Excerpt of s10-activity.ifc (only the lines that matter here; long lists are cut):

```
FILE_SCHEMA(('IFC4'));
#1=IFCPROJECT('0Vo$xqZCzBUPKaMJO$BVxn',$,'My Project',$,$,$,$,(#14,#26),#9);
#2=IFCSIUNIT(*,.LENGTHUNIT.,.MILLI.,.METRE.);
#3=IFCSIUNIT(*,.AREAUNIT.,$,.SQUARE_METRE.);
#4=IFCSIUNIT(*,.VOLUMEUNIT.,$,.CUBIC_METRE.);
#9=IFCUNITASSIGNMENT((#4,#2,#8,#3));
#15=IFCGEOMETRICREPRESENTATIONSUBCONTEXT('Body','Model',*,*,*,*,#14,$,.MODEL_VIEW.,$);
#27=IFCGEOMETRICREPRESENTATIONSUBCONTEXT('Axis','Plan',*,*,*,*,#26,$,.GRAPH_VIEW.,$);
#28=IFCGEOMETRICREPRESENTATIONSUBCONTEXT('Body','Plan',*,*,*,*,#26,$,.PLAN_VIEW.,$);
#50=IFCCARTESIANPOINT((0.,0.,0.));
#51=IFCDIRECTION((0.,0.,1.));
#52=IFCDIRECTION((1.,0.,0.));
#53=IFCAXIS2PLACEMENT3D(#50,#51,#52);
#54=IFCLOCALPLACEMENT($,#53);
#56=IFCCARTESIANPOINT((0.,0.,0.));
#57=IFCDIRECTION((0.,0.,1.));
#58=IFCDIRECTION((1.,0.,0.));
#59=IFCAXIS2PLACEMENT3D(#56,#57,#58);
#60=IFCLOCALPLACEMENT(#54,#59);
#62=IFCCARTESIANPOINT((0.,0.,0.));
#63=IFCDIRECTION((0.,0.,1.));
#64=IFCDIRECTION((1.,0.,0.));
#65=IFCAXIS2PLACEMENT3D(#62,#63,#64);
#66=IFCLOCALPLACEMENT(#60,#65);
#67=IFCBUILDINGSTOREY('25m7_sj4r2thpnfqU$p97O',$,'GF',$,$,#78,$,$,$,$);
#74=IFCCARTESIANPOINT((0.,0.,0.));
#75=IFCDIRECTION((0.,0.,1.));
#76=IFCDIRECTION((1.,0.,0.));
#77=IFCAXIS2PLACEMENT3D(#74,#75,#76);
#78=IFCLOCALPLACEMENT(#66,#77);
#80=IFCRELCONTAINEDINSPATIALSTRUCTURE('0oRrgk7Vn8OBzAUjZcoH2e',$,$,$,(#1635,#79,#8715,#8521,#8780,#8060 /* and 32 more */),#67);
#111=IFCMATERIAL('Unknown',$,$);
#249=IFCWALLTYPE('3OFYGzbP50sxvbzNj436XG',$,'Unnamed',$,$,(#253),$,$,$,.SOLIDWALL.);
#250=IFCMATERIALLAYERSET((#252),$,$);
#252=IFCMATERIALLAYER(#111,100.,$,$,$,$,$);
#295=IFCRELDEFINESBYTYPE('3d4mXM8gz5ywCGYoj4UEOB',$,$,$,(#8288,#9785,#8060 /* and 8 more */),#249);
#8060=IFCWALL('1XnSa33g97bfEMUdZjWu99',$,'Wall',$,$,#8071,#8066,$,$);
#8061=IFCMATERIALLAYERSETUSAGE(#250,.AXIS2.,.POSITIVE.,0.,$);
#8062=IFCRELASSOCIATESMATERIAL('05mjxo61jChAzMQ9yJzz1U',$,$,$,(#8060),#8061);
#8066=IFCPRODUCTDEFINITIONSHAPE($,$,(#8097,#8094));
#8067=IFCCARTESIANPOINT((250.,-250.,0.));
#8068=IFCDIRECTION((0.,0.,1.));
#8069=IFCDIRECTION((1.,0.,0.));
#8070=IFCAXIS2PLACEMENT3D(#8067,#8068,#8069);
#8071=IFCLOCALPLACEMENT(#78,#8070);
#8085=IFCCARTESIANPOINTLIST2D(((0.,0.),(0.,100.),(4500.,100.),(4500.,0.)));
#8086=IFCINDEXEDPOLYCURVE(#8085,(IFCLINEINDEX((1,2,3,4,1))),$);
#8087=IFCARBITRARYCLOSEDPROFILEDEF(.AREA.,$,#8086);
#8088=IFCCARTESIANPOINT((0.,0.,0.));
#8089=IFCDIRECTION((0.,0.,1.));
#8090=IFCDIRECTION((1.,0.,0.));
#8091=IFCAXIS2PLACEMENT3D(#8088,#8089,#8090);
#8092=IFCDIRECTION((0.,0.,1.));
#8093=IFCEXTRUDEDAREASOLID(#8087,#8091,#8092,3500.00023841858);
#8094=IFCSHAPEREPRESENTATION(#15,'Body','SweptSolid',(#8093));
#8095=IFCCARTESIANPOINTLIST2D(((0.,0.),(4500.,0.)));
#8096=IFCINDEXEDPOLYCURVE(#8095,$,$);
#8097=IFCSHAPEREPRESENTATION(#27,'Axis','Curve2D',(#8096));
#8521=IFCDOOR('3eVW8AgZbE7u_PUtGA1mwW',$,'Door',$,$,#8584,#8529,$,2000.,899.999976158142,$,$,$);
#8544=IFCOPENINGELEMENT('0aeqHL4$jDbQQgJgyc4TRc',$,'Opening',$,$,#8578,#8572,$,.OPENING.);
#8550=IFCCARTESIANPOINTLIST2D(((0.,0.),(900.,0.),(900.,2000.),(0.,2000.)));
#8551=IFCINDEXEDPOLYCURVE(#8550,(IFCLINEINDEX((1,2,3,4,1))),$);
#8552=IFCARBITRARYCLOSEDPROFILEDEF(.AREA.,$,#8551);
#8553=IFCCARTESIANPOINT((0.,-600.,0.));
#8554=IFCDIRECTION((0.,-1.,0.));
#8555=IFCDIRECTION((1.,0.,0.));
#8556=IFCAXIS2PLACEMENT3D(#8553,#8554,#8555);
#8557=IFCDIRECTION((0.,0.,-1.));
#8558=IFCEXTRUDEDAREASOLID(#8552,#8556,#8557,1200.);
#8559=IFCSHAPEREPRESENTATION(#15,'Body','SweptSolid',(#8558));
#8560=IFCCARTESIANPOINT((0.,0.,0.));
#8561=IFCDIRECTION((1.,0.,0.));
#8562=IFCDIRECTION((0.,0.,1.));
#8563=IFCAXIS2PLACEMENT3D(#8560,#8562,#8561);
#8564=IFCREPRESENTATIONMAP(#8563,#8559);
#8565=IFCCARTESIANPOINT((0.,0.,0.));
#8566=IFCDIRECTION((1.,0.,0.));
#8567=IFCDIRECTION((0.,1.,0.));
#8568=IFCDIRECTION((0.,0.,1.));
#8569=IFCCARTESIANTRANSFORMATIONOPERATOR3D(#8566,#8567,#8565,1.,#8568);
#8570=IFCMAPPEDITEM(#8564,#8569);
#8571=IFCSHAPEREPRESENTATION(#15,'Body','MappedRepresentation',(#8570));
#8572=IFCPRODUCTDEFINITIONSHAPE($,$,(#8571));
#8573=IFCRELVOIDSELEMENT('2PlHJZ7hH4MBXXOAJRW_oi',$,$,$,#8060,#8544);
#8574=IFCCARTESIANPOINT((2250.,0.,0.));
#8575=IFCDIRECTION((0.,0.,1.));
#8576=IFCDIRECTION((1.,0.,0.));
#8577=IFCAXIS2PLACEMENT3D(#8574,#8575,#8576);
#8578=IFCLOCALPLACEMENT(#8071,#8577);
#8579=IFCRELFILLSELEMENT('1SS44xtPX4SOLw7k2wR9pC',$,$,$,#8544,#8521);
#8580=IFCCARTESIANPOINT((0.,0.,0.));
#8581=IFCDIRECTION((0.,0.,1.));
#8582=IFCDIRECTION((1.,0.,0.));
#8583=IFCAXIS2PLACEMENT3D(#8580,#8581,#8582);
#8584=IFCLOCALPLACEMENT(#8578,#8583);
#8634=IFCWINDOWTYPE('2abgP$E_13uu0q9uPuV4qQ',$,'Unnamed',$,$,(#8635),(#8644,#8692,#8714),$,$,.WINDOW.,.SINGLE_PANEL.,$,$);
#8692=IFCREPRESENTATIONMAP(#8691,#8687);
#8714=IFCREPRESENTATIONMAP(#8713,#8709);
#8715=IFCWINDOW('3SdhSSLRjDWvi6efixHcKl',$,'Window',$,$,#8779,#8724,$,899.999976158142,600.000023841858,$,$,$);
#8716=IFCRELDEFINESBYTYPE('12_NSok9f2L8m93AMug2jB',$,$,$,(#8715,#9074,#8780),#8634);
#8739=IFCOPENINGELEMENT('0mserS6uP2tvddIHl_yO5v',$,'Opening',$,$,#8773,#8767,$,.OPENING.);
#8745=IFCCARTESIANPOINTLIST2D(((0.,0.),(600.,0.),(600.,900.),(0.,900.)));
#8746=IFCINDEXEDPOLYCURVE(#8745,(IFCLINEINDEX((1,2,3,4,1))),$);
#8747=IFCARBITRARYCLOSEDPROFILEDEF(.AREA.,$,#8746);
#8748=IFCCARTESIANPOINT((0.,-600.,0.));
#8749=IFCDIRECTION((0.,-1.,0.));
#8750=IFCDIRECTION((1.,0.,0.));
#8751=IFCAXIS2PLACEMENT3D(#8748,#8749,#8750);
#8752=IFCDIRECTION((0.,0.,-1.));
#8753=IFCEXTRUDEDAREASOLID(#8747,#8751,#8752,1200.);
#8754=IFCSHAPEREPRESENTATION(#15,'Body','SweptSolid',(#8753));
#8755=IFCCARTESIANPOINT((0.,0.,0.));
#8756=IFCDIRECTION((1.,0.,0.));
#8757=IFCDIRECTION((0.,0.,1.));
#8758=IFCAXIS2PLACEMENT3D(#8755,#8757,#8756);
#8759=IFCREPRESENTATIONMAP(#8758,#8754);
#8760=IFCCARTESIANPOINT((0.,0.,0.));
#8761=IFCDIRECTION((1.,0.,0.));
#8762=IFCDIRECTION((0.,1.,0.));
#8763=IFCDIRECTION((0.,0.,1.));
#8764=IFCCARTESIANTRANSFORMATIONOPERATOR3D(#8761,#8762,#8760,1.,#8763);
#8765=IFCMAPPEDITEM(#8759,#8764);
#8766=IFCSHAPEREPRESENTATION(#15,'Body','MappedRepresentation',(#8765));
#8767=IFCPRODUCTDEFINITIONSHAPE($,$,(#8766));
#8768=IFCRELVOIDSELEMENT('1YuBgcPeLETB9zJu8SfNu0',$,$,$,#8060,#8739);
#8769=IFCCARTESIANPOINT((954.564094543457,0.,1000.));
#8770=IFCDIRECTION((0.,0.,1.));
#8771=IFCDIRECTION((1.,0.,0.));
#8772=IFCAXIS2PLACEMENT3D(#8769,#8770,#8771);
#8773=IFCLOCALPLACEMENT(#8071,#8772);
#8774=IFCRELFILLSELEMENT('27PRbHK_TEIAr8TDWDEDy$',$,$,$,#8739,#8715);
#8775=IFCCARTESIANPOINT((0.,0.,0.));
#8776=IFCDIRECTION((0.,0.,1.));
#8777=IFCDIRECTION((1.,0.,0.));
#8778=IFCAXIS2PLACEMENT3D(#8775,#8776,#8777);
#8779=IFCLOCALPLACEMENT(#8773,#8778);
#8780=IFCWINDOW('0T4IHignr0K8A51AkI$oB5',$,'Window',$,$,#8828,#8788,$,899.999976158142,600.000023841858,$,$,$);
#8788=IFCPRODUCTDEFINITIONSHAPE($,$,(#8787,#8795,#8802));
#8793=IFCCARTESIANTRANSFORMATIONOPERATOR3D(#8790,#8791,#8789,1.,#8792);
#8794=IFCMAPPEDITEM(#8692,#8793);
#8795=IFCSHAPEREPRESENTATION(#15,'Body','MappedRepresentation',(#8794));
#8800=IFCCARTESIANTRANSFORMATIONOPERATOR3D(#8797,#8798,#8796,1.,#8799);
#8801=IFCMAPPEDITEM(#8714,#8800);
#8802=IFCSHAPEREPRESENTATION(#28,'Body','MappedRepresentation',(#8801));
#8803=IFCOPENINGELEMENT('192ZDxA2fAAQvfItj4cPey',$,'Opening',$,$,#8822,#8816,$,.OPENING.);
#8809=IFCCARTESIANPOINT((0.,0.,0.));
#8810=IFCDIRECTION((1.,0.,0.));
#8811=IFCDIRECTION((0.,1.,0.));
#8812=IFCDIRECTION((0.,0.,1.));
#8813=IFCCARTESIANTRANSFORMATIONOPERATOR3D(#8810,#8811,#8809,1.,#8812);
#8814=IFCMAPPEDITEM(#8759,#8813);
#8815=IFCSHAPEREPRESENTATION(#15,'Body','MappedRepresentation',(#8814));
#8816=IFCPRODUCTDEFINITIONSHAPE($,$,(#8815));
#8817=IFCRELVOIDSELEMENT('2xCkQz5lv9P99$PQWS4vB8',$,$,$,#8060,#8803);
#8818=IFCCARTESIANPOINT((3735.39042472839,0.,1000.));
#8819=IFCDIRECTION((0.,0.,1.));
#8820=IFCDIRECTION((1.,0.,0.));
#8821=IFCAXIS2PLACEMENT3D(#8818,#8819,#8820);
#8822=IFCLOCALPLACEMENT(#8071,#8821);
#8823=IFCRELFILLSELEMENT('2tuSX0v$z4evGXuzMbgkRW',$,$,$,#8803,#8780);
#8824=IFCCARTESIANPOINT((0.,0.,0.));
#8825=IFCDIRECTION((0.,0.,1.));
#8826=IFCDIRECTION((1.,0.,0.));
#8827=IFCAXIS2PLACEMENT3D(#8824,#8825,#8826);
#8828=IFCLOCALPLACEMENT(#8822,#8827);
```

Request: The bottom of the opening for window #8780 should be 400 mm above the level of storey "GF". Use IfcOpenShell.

```python
import numpy as np
import ifcopenshell
import ifcopenshell.api.geometry
import ifcopenshell.geom
import ifcopenshell.util.element
import ifcopenshell.util.placement
import ifcopenshell.util.shape
import ifcopenshell.util.unit

model = ifcopenshell.open("s10-activity.ifc")
unit_scale = ifcopenshell.util.unit.calculate_unit_scale(model)

window = model.by_guid("0T4IHignr0K8A51AkI$oB5")
opening = window.FillsVoids[0].RelatingOpeningElement
storey = ifcopenshell.util.element.get_container(window, ifc_class="IfcBuildingStorey")
level = ifcopenshell.util.placement.get_local_placement(storey.ObjectPlacement)[2, 3]

# The opening's origin need not be at the sill, so measure its lowest point.
shape = ifcopenshell.geom.create_shape(ifcopenshell.geom.settings(), opening)
bottom = ifcopenshell.util.shape.get_shape_bottom_elevation(shape, shape.geometry) / unit_scale
dz = level + 0.4 / unit_scale - bottom

shift = np.array([0.0, 0.0, dz])
# The window is placed relative to its opening, so it follows when the opening moves.
matrix = ifcopenshell.util.placement.get_local_placement(opening.ObjectPlacement)
matrix[:3, 3] += shift
ifcopenshell.api.geometry.edit_object_placement(
    model, product=opening, matrix=matrix, is_si=False, should_transform_children=True
)

print(f"moved by {dz * unit_scale:+.3f} m")

model.write("s10-activity_v2.ifc")
```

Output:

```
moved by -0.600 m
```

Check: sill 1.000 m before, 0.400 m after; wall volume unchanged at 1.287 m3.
